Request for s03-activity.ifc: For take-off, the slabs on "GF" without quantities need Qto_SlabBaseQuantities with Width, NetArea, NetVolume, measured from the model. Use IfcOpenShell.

First a look at what the model holds.

```python
import ifcopenshell
import ifcopenshell.util.element
import ifcopenshell.util.unit

model = ifcopenshell.open("s03-activity.ifc")
print(model.schema)
for unit_type in ("LENGTHUNIT", "AREAUNIT", "VOLUMEUNIT"):
    print(unit_type, ifcopenshell.util.unit.calculate_unit_scale(model, unit_type))
storey = next(s for s in model.by_type("IfcBuildingStorey") if s.Name == "GF")
slabs = [e for e in ifcopenshell.util.element.get_decomposition(storey) if e.is_a("IfcSlab")]
for e in sorted(slabs, key=lambda e: e.id()):
    print(e.id(), e.is_a(), e.Name, list(ifcopenshell.util.element.get_psets(e, qtos_only=True)), sep=" | ")
```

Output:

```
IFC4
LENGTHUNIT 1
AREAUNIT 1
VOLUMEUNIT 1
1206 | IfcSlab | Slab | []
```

```python
import ifcopenshell
import ifcopenshell.api.pset
import ifcopenshell.geom
import ifcopenshell.util.element
import ifcopenshell.util.shape
import ifcopenshell.util.unit

model = ifcopenshell.open("s03-activity.ifc")
unit_scale = ifcopenshell.util.unit.calculate_unit_scale(model)
area_scale = ifcopenshell.util.unit.calculate_unit_scale(model, "AREAUNIT")
volume_scale = ifcopenshell.util.unit.calculate_unit_scale(model, "VOLUMEUNIT")
settings = ifcopenshell.geom.settings()

storey = next(s for s in model.by_type("IfcBuildingStorey") if s.Name == "GF")
slabs = [e for e in ifcopenshell.util.element.get_decomposition(storey) if e.is_a("IfcSlab")]

for e in sorted(slabs, key=lambda e: e.id()):
    if ifcopenshell.util.element.get_psets(e, qtos_only=True, should_inherit=False):
        continue
    # Geometry comes back in metres, in the element's own axes.
    shape = ifcopenshell.geom.create_shape(settings, e)
    values = {
        "Width": ifcopenshell.util.shape.get_z(shape.geometry) / unit_scale,
        "NetArea": ifcopenshell.util.shape.get_footprint_area(shape.geometry) / area_scale,
        "NetVolume": ifcopenshell.util.shape.get_volume(shape.geometry) / volume_scale,
    }
    qto = ifcopenshell.api.pset.add_qto(model, product=e, name="Qto_SlabBaseQuantities")
    ifcopenshell.api.pset.edit_qto(model, qto=qto, properties=values)
    print(e.id(), {k: round(v, 3) for k, v in values.items()})

model.write("s03-activity_v2.ifc")
```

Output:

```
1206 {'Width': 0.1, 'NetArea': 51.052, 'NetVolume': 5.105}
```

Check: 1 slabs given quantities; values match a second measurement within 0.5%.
